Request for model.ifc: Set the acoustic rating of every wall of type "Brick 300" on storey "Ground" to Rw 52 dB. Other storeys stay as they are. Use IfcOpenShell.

First a look at what the model holds.

```python
import ifcopenshell
import ifcopenshell.util.element

model = ifcopenshell.open("model.ifc")
print(model.schema)
storey = next(s for s in model.by_type("IfcBuildingStorey") if s.Name == "Ground")
walls = [e for e in ifcopenshell.util.element.get_decomposition(storey) if e.is_a("IfcWall")]
seen = {}
for e in walls:
    element_type = ifcopenshell.util.element.get_type(e)
    key = (element_type.Name if element_type != e and element_type else None, ifcopenshell.util.element.get_pset(e, "Pset_WallCommon", "AcousticRating"))
    seen[key] = seen.get(key, 0) + 1
for (name, value), count in sorted(seen.items(), key=str):
    print(count, "x", name, "|", value)
```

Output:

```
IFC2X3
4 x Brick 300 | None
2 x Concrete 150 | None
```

```python
import ifcopenshell
import ifcopenshell.api.pset
import ifcopenshell.util.element

model = ifcopenshell.open("model.ifc")

storey = next(s for s in model.by_type("IfcBuildingStorey") if s.Name == "Ground")
walls = [e for e in ifcopenshell.util.element.get_decomposition(storey) if e.is_a("IfcWall")]

count = 0
for e in walls:
    element_type = ifcopenshell.util.element.get_type(e)
    if element_type in (None, e) or element_type.Name != "Brick 300":
        continue
    # add_pset returns the element's existing set when there is one.
    pset = ifcopenshell.api.pset.add_pset(model, product=e, name="Pset_WallCommon")
    ifcopenshell.api.pset.edit_pset(model, pset=pset, properties={"AcousticRating": "Rw 52 dB"})
    count += 1

print(count, "walls updated")

model.write("model-out.ifc")
```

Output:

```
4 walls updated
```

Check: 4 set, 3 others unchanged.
